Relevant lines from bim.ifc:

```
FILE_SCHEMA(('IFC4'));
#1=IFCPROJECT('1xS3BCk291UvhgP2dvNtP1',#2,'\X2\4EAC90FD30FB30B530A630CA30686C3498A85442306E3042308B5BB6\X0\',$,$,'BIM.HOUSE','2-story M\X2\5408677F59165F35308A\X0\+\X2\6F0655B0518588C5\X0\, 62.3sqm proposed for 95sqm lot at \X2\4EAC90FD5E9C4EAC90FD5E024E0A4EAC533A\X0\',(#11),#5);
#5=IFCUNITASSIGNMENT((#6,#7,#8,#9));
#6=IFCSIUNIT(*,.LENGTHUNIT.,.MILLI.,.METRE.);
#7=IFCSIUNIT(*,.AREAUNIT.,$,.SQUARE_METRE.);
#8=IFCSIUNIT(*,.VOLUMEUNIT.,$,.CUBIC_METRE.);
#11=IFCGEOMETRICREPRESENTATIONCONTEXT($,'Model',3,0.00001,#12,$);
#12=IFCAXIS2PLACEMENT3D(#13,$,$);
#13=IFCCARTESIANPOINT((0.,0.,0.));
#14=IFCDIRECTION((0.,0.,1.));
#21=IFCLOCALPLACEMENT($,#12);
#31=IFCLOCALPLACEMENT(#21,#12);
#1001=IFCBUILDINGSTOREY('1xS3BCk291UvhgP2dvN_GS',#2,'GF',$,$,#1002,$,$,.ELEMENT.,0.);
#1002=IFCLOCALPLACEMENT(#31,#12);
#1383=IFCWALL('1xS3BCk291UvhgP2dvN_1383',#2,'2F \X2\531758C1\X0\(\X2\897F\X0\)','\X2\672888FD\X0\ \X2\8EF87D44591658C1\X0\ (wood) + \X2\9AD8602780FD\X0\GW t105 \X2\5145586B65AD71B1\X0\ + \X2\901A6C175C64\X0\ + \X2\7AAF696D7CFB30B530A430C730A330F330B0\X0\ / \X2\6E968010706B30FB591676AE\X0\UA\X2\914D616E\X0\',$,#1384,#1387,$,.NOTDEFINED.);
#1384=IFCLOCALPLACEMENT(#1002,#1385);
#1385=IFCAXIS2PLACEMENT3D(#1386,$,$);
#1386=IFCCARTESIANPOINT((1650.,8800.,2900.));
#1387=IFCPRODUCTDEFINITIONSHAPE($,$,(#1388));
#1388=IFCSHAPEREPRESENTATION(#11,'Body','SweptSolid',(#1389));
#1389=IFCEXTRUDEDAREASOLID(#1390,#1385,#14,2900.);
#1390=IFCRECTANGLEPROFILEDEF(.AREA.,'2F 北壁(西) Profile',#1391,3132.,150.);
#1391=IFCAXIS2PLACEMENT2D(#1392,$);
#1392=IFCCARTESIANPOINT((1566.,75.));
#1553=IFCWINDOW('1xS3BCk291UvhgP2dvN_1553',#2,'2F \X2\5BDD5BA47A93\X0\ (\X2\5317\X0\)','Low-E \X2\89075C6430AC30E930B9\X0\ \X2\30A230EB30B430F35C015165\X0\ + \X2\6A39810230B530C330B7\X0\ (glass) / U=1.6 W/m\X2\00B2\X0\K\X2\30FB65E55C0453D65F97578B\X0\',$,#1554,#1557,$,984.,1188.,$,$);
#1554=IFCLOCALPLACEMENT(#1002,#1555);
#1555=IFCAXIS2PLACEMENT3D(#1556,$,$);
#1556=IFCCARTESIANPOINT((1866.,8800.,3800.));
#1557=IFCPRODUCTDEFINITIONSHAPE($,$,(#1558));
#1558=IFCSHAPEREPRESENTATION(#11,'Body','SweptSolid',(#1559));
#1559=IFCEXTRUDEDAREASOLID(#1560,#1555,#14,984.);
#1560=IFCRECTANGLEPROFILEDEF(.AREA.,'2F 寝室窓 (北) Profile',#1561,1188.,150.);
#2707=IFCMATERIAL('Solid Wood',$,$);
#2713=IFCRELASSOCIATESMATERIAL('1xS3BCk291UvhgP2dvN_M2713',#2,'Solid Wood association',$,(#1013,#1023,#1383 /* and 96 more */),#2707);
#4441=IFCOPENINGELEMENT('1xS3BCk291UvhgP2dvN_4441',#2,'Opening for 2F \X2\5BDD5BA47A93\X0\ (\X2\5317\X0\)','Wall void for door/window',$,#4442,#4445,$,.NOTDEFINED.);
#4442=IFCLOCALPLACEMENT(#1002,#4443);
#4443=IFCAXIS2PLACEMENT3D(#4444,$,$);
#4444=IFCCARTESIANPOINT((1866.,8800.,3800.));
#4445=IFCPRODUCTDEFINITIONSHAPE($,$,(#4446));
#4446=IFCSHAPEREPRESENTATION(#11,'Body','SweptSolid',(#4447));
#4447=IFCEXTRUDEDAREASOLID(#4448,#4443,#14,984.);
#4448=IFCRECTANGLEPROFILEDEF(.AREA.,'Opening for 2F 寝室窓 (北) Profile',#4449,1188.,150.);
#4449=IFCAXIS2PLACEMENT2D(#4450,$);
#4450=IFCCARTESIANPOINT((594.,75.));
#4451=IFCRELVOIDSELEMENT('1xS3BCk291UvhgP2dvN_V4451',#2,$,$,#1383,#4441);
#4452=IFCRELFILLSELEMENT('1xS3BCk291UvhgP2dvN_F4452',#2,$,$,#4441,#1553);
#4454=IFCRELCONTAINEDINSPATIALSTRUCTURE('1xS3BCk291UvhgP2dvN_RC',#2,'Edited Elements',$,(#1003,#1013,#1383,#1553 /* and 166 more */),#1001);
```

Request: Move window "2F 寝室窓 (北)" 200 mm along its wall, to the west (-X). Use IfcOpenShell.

```python
import ifcopenshell
import ifcopenshell.api.geometry
import ifcopenshell.util.placement

model = ifcopenshell.open("bim.ifc")

window = model.by_guid("1xS3BCk291UvhgP2dvN_1553")
opening = window.FillsVoids[0].RelatingOpeningElement
wall = opening.VoidsElements[0].RelatingBuildingElement

wall_matrix = ifcopenshell.util.placement.get_local_placement(wall.ObjectPlacement)
shift = wall_matrix[:3, 0] * -200.0
before = ifcopenshell.util.placement.get_local_placement(window.ObjectPlacement)[:3, 3].copy()

# The window is not placed relative to its opening, so move both.
for product in (opening, window):
    matrix = ifcopenshell.util.placement.get_local_placement(product.ObjectPlacement)
    matrix[:3, 3] += shift
    ifcopenshell.api.geometry.edit_object_placement(model, product=product, matrix=matrix, is_si=False)

after = ifcopenshell.util.placement.get_local_placement(window.ObjectPlacement)[:3, 3]
print("window moved by", (after - before).round(3) + 0.0)

model.write("bim_rev.ifc")
```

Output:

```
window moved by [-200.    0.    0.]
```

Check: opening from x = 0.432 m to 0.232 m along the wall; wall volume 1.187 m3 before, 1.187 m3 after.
